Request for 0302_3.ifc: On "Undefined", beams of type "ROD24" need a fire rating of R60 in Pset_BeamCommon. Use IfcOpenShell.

First a look at what the model holds.

```python
import ifcopenshell
import ifcopenshell.util.element

model = ifcopenshell.open("0302_3.ifc")
print(model.schema)
storey = next(s for s in model.by_type("IfcBuildingStorey") if s.Name == "Undefined")
beams = [e for e in ifcopenshell.util.element.get_decomposition(storey) if e.is_a("IfcBeam")]
seen = {}
for e in beams:
    element_type = ifcopenshell.util.element.get_type(e)
    key = (element_type.Name if element_type != e and element_type else None, ifcopenshell.util.element.get_pset(e, "Pset_BeamCommon", "FireRating"))
    seen[key] = seen.get(key, 0) + 1
for (name, value), count in sorted(seen.items(), key=str):
    print(count, "x", name, "|", value)
```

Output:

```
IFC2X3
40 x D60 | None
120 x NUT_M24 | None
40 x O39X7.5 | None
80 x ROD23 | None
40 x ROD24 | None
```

```python
import ifcopenshell
import ifcopenshell.api.pset
import ifcopenshell.util.element

model = ifcopenshell.open("0302_3.ifc")

storey = next(s for s in model.by_type("IfcBuildingStorey") if s.Name == "Undefined")
beams = [e for e in ifcopenshell.util.element.get_decomposition(storey) if e.is_a("IfcBeam")]

count = 0
for e in beams:
    element_type = ifcopenshell.util.element.get_type(e)
    if element_type in (None, e) or element_type.Name != "ROD24":
        continue
    found = ifcopenshell.util.element.get_pset(e, "Pset_BeamCommon", should_inherit=False)
    if found:
        pset = model.by_id(found["id"])
        if len(ifcopenshell.util.element.get_elements_by_pset(pset)) > 1:
            pset = ifcopenshell.api.pset.unshare_pset(model, products=[e], pset=pset)[0]
    else:
        pset = ifcopenshell.api.pset.add_pset(model, product=e, name="Pset_BeamCommon")
    ifcopenshell.api.pset.edit_pset(model, pset=pset, properties={"FireRating": "R60"})
    count += 1

print(count, "beams updated")

model.write("0302_3_edited.ifc")
```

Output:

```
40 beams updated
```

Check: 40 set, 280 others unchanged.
